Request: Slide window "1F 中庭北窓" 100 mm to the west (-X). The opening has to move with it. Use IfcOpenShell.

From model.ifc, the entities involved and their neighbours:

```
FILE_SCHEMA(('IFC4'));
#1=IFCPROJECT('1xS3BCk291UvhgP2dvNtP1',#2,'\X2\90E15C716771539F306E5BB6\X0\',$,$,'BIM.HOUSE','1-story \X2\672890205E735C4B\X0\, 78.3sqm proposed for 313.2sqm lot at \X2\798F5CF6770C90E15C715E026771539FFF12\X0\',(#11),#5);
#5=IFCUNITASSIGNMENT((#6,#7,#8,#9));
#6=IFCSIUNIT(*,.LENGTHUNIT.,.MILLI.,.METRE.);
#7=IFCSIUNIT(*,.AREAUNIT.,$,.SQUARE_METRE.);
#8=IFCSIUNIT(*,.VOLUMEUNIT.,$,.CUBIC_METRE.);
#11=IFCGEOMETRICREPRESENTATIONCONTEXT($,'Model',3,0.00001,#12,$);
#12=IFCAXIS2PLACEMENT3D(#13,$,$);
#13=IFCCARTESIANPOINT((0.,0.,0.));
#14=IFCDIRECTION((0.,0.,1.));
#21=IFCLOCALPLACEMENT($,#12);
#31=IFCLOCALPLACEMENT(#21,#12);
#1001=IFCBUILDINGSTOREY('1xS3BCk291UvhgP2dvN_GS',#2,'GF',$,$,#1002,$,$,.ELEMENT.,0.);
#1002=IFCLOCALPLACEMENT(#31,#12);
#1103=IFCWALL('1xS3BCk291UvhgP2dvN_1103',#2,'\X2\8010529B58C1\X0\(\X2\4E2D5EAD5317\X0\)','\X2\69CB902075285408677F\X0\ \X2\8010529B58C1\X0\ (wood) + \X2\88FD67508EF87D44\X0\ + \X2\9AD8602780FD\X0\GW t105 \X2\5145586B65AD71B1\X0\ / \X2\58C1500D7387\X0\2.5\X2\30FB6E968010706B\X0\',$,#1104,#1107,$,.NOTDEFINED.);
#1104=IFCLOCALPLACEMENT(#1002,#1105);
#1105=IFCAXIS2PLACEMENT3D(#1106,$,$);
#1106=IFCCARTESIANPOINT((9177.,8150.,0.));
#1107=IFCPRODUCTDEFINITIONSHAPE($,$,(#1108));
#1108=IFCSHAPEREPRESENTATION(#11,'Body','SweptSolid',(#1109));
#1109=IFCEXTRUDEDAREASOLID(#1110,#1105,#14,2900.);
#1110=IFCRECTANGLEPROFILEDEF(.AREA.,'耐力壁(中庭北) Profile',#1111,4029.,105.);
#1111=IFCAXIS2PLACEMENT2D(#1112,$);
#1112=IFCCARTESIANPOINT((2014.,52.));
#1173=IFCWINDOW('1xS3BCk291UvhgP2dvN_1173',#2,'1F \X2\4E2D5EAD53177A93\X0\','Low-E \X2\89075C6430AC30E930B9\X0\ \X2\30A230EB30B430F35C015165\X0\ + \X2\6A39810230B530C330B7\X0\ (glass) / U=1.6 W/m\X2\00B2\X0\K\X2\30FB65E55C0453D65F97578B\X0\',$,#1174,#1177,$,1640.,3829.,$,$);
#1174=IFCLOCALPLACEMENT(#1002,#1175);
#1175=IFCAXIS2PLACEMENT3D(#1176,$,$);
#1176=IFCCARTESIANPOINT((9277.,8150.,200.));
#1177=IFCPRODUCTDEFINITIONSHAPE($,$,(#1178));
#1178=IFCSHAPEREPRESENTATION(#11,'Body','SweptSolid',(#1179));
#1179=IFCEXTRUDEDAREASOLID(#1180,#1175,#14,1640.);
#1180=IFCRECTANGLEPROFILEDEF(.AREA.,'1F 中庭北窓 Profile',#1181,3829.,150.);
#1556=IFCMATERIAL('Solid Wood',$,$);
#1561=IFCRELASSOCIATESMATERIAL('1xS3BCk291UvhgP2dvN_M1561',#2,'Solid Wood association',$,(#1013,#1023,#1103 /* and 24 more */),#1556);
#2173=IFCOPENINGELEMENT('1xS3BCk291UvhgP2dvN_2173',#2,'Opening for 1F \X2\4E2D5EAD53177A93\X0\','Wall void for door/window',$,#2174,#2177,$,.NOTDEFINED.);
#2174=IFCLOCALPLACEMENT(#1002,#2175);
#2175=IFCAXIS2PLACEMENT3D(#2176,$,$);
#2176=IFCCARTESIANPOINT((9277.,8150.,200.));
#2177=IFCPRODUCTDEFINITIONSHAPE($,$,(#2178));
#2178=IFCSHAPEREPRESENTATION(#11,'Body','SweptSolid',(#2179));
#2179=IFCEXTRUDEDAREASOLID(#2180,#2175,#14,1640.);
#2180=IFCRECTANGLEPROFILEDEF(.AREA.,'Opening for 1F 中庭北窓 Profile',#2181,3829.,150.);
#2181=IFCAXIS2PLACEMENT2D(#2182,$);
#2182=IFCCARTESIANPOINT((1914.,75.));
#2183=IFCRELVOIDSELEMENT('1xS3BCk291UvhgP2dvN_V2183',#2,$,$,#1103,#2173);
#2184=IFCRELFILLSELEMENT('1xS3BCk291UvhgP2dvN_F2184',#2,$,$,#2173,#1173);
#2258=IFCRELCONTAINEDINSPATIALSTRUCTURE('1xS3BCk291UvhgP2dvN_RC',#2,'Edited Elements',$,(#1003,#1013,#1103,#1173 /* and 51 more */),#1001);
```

```python
import ifcopenshell
import ifcopenshell.api.geometry
import ifcopenshell.util.placement

model = ifcopenshell.open("model.ifc")

window = model.by_guid("1xS3BCk291UvhgP2dvN_1173")
opening = window.FillsVoids[0].RelatingOpeningElement
wall = opening.VoidsElements[0].RelatingBuildingElement

wall_matrix = ifcopenshell.util.placement.get_local_placement(wall.ObjectPlacement)
shift = wall_matrix[:3, 0] * -100.0
before = ifcopenshell.util.placement.get_local_placement(window.ObjectPlacement)[:3, 3].copy()

# The window is not placed relative to its opening, so move both.
for product in (opening, window):
    matrix = ifcopenshell.util.placement.get_local_placement(product.ObjectPlacement)
    matrix[:3, 3] += shift
    ifcopenshell.api.geometry.edit_object_placement(model, product=product, matrix=matrix, is_si=False)

after = ifcopenshell.util.placement.get_local_placement(window.ObjectPlacement)[:3, 3]
print("window moved by", (after - before).round(3) + 0.0)

model.write("model_rev.ifc")
```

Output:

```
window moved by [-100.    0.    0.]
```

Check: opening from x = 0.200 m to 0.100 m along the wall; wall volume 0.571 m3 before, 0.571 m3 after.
